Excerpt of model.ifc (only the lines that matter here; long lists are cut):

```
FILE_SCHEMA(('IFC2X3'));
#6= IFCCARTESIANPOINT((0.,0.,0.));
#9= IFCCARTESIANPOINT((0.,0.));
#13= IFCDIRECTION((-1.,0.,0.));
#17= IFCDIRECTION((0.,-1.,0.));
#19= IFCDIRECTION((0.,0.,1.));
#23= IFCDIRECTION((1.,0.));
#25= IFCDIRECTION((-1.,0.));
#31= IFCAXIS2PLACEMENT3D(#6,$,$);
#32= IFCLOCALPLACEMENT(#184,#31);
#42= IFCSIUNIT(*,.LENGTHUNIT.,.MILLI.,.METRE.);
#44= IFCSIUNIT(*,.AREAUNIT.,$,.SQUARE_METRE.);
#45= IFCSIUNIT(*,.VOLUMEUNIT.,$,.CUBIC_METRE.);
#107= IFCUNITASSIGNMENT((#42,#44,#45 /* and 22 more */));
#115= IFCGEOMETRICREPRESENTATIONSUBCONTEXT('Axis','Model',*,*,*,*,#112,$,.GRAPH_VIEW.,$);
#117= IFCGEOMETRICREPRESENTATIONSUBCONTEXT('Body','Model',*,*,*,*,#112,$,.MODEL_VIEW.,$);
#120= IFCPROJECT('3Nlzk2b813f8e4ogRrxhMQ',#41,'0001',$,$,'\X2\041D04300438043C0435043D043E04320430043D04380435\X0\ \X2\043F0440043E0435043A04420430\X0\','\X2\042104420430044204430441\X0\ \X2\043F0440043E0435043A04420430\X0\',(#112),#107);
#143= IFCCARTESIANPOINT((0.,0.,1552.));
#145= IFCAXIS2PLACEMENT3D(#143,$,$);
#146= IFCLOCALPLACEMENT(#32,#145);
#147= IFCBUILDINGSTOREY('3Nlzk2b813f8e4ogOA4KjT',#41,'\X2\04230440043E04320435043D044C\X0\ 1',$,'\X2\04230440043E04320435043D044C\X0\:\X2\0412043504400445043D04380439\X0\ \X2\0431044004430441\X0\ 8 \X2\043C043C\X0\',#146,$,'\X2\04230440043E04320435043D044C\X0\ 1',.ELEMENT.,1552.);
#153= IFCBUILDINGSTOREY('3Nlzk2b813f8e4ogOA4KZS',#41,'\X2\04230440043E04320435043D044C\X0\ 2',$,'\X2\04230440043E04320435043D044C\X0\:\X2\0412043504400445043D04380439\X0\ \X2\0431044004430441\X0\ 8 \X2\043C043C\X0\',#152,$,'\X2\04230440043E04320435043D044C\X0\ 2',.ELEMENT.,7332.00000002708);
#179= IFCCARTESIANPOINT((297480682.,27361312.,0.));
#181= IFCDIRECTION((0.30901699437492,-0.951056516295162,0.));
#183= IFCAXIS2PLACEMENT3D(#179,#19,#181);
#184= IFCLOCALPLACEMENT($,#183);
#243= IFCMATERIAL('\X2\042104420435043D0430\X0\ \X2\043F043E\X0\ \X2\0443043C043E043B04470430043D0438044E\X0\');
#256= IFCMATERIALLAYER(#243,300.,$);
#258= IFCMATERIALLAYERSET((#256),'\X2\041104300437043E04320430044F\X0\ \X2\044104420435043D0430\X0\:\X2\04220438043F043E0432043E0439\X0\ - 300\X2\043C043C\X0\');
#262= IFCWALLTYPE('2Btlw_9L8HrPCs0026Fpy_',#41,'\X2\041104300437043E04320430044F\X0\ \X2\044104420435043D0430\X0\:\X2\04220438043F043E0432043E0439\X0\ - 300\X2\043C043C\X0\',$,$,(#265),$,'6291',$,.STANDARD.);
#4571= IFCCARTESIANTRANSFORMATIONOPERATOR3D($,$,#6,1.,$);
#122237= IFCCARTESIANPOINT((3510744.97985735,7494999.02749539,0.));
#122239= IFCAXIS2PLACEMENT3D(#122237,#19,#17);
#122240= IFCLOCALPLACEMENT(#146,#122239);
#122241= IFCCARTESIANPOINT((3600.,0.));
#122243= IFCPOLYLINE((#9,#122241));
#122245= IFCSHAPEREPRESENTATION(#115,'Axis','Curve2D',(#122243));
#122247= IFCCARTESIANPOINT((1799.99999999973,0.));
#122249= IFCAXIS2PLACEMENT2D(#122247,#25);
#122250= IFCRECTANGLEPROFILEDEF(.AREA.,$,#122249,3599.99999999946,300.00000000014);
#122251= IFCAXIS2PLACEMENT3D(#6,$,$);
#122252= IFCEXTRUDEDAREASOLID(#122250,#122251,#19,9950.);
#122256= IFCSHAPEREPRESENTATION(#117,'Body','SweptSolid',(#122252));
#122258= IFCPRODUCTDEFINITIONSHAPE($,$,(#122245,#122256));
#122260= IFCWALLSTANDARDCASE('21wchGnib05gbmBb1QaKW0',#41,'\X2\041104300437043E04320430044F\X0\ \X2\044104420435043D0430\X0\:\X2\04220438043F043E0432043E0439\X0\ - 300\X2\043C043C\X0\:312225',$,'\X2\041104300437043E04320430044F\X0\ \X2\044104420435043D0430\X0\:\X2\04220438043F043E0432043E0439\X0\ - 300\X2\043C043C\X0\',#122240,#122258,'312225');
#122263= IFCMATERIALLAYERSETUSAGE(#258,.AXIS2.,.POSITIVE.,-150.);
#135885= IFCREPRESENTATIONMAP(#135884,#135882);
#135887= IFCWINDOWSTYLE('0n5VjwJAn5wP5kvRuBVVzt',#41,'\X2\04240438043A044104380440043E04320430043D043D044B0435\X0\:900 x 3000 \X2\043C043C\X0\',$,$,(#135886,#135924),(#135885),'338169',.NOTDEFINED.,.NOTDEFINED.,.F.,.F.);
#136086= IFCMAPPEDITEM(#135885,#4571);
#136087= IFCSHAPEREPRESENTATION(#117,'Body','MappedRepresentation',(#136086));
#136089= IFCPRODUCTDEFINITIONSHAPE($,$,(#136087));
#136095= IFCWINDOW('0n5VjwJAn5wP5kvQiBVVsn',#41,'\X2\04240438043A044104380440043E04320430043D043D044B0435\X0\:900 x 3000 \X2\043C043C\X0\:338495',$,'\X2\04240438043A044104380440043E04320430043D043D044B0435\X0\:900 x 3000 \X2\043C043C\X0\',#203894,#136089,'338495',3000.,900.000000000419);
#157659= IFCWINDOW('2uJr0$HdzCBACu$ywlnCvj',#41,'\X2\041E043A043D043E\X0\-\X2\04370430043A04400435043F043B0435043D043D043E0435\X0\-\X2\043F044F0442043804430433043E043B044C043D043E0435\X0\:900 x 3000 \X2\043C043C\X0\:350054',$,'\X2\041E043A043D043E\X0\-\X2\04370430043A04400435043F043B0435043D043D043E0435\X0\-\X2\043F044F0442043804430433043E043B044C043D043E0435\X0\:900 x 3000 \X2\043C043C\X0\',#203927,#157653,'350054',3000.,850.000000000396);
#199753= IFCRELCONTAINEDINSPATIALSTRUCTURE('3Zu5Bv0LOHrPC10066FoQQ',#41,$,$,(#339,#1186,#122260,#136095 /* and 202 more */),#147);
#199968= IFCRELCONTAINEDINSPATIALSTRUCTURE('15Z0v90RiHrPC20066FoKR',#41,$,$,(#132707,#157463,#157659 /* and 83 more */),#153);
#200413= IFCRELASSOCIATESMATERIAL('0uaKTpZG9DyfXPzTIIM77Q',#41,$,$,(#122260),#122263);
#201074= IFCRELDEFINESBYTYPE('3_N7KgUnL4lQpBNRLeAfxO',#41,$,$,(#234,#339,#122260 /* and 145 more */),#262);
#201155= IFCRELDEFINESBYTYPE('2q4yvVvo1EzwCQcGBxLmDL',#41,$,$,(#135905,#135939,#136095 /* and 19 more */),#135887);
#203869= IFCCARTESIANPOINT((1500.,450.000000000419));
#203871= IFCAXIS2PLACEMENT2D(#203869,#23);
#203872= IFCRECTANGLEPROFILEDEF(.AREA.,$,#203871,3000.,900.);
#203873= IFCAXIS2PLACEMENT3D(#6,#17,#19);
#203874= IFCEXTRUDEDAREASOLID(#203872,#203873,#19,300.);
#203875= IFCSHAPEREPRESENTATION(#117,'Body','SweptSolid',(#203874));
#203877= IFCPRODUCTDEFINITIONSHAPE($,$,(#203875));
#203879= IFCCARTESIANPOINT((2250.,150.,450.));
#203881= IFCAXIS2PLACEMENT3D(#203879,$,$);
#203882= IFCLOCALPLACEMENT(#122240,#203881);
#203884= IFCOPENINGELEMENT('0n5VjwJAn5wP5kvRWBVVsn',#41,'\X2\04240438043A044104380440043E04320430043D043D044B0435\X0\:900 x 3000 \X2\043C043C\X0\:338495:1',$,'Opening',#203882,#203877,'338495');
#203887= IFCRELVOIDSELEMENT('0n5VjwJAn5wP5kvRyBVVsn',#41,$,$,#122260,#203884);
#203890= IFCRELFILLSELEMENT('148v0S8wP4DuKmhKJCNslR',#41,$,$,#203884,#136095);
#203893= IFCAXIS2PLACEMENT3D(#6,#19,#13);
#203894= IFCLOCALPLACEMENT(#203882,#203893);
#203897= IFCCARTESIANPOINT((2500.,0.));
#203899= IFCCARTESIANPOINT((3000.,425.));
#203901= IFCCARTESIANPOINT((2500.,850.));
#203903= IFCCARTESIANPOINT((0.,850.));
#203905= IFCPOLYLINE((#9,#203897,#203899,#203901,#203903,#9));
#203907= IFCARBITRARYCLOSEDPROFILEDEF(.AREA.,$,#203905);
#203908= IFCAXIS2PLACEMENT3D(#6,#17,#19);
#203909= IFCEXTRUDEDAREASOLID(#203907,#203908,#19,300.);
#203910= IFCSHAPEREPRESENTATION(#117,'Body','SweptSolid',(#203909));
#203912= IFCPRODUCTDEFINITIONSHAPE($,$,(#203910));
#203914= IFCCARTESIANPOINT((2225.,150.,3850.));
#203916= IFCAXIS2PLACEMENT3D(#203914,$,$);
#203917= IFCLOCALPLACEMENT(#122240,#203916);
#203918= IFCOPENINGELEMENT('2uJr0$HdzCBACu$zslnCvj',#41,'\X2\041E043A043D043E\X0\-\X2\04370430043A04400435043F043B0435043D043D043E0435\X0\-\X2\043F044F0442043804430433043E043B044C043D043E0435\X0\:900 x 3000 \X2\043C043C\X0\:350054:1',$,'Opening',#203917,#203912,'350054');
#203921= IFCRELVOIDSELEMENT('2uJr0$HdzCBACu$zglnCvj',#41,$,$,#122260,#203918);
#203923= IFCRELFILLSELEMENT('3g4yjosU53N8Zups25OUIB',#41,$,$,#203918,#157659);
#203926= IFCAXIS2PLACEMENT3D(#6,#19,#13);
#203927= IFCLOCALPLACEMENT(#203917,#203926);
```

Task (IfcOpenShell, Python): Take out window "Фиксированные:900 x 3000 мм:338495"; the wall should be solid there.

```python
import ifcopenshell
import ifcopenshell.api.feature
import ifcopenshell.api.root
import ifcopenshell.geom
import ifcopenshell.util.shape

model = ifcopenshell.open("model.ifc")
settings = ifcopenshell.geom.settings()


def volume(element):
    """Net volume in cubic metres, openings subtracted."""
    shape = ifcopenshell.geom.create_shape(settings, element)
    return ifcopenshell.util.shape.get_volume(shape.geometry)


window = model.by_guid("0n5VjwJAn5wP5kvQiBVVsn")
opening = window.FillsVoids[0].RelatingOpeningElement
wall = opening.VoidsElements[0].RelatingBuildingElement
before = volume(wall)

ifcopenshell.api.root.remove_product(model, product=window)
ifcopenshell.api.feature.remove_feature(model, feature=opening)

after = volume(wall)

print(f"wall volume {before:.3f} -> {after:.3f} m3")

model.write("model_edited.ifc")
```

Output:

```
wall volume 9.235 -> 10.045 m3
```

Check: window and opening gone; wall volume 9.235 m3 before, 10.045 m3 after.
